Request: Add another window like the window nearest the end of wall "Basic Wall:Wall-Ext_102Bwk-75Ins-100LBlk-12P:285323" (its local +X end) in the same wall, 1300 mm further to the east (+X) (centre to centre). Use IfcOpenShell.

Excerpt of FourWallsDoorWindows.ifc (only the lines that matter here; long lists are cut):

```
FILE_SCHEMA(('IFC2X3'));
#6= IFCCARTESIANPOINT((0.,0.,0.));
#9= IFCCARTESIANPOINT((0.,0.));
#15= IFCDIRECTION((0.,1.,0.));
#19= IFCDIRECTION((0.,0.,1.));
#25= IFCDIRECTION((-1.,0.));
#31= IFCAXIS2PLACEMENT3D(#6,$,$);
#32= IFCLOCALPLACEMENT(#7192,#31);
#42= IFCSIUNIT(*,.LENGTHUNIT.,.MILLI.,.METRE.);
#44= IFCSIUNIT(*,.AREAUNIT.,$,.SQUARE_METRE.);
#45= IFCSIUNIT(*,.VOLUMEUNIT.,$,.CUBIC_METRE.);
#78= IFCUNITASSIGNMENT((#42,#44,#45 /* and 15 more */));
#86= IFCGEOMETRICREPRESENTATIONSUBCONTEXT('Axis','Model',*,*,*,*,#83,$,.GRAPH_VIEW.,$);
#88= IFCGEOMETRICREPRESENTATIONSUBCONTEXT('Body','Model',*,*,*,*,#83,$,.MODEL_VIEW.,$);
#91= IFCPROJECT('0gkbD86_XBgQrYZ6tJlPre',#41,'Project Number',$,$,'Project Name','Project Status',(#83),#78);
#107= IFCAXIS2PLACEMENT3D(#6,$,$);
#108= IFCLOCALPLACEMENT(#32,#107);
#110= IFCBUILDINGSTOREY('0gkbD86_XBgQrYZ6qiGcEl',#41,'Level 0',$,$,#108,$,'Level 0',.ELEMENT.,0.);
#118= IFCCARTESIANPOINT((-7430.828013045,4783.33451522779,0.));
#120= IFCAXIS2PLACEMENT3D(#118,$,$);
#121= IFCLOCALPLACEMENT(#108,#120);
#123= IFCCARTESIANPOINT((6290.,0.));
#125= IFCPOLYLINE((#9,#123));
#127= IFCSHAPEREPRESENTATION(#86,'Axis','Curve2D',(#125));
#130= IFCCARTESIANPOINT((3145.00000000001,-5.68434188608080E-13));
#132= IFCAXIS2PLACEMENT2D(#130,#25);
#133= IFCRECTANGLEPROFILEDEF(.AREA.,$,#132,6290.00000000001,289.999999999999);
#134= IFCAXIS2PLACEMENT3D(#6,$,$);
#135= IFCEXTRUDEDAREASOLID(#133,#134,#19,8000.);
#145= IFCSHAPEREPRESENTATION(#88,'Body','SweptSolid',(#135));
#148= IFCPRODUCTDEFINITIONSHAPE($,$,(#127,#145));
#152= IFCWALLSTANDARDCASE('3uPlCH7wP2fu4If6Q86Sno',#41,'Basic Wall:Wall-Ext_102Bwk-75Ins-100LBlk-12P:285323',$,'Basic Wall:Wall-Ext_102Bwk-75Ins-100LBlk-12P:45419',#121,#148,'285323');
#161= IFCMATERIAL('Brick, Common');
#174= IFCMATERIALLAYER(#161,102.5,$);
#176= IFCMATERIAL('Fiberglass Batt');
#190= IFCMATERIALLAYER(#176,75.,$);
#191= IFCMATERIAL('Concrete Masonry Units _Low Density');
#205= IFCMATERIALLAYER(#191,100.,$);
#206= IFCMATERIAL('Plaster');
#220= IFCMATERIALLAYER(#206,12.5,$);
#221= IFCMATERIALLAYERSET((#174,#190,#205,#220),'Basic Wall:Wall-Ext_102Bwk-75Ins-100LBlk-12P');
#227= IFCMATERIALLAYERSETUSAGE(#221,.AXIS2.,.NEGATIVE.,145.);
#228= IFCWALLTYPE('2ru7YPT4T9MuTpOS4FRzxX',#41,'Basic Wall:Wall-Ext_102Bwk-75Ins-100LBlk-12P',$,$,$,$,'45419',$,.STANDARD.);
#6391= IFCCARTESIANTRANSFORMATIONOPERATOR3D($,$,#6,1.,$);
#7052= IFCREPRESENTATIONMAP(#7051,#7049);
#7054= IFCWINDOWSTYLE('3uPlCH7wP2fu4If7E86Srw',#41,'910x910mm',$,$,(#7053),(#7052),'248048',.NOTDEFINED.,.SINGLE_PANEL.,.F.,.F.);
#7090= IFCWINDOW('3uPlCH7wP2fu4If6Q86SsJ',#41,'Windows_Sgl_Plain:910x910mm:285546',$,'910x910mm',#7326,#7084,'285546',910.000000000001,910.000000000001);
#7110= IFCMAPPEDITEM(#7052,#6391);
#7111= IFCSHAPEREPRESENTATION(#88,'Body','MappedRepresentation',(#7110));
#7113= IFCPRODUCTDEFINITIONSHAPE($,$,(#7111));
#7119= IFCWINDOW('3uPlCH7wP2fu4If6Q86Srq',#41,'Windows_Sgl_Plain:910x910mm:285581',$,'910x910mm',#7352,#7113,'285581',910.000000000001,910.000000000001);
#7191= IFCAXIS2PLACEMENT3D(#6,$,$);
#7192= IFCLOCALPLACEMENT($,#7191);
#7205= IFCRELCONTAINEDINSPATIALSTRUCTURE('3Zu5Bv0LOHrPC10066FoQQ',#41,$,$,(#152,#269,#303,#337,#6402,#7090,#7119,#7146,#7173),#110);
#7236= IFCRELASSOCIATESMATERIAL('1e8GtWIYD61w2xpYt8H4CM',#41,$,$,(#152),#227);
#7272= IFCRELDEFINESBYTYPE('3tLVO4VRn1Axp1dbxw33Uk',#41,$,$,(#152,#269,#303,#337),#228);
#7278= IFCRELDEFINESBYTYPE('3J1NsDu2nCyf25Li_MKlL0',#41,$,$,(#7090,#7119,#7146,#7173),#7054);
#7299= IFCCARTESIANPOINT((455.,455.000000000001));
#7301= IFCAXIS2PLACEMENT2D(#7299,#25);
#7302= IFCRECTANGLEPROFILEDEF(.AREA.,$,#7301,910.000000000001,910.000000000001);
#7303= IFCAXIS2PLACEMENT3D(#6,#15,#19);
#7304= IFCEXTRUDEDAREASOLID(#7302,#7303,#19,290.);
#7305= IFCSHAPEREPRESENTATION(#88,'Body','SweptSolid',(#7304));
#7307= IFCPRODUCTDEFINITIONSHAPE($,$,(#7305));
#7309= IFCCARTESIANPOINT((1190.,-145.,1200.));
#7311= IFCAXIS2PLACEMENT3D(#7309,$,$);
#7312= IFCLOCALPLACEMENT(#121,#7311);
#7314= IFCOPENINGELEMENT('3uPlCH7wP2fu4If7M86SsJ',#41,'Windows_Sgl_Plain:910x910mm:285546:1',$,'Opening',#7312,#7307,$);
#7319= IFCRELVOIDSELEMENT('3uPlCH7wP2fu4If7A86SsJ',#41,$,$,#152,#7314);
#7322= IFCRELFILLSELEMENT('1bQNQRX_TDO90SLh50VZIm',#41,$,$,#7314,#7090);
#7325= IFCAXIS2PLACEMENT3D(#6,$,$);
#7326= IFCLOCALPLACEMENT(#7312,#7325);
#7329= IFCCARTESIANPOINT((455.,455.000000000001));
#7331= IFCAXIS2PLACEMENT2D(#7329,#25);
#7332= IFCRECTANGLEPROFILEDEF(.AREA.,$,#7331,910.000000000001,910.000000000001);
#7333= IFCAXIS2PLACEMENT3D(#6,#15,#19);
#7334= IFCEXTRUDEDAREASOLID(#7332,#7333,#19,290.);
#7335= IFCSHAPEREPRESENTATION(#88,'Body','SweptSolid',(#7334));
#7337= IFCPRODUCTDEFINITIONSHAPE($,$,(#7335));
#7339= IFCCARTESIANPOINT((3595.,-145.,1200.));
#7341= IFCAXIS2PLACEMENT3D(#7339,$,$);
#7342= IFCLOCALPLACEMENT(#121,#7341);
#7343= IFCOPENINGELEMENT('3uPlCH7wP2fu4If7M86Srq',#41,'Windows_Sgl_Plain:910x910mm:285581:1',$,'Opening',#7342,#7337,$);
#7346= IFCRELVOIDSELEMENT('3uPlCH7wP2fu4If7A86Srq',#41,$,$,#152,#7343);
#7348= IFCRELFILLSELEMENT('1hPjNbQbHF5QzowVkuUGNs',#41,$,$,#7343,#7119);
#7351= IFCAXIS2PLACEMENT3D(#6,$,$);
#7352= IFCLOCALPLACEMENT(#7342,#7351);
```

```python
import ifcopenshell
import ifcopenshell.api.feature
import ifcopenshell.api.geometry
import ifcopenshell.api.root
import ifcopenshell.geom
import ifcopenshell.util.element
import ifcopenshell.util.placement
import ifcopenshell.util.shape
import ifcopenshell.util.unit

model = ifcopenshell.open("FourWallsDoorWindows.ifc")
unit_scale = ifcopenshell.util.unit.calculate_unit_scale(model)
settings = ifcopenshell.geom.settings()


def volume(element):
    """Net volume in cubic metres, openings subtracted."""
    shape = ifcopenshell.geom.create_shape(settings, element)
    return ifcopenshell.util.shape.get_volume(shape.geometry)


def reuse_history(source, copy):
    """copy_class also copies each property set's owner history, people and application; keep the originals."""
    for rel in copy.IsDefinedBy:
        if rel.is_a("IfcRelDefinesByProperties") and (history := rel.RelatingPropertyDefinition.OwnerHistory):
            rel.RelatingPropertyDefinition.OwnerHistory = source.OwnerHistory
            ifcopenshell.util.element.remove_deep2(model, history)


window = model.by_guid("3uPlCH7wP2fu4If6Q86Srq")
opening = window.FillsVoids[0].RelatingOpeningElement
wall = opening.VoidsElements[0].RelatingBuildingElement
before = volume(wall)
shift = ifcopenshell.util.placement.get_local_placement(wall.ObjectPlacement)[:3, 0] * 1.3 / unit_scale

# copy_class copies the void relationship, type, container and properties, but no geometry.
new_opening = ifcopenshell.api.root.copy_class(model, product=opening)
new_opening.Representation = ifcopenshell.util.element.copy_deep(
    model, opening.Representation, exclude=["IfcGeometricRepresentationContext", "IfcRepresentationMap"]
)
new_opening.Name = "Windows_Sgl_Plain:910x910mm"
new_window = ifcopenshell.api.root.copy_class(model, product=window)
new_window.Representation = ifcopenshell.util.element.copy_deep(
    model, window.Representation, exclude=["IfcGeometricRepresentationContext", "IfcRepresentationMap"]
)
new_window.Name = "Windows_Sgl_Plain:910x910mm"
new_window.Tag = None
reuse_history(window, new_window)
fills = ifcopenshell.api.feature.add_filling(model, opening=new_opening, element=new_window)
fills.OwnerHistory = new_window.OwnerHistory  # required in IFC2X3

for old, new in ((opening, new_opening), (window, new_window)):
    matrix = ifcopenshell.util.placement.get_local_placement(old.ObjectPlacement)
    matrix[:3, 3] += shift
    ifcopenshell.api.geometry.edit_object_placement(model, product=new, matrix=matrix, is_si=False)

after = volume(wall)

print(f"wall volume {before:.3f} -> {after:.3f} m3")

model.write("FourWallsDoorWindows_edited.ifc")
```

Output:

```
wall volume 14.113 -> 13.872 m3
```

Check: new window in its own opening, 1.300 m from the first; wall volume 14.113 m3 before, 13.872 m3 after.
